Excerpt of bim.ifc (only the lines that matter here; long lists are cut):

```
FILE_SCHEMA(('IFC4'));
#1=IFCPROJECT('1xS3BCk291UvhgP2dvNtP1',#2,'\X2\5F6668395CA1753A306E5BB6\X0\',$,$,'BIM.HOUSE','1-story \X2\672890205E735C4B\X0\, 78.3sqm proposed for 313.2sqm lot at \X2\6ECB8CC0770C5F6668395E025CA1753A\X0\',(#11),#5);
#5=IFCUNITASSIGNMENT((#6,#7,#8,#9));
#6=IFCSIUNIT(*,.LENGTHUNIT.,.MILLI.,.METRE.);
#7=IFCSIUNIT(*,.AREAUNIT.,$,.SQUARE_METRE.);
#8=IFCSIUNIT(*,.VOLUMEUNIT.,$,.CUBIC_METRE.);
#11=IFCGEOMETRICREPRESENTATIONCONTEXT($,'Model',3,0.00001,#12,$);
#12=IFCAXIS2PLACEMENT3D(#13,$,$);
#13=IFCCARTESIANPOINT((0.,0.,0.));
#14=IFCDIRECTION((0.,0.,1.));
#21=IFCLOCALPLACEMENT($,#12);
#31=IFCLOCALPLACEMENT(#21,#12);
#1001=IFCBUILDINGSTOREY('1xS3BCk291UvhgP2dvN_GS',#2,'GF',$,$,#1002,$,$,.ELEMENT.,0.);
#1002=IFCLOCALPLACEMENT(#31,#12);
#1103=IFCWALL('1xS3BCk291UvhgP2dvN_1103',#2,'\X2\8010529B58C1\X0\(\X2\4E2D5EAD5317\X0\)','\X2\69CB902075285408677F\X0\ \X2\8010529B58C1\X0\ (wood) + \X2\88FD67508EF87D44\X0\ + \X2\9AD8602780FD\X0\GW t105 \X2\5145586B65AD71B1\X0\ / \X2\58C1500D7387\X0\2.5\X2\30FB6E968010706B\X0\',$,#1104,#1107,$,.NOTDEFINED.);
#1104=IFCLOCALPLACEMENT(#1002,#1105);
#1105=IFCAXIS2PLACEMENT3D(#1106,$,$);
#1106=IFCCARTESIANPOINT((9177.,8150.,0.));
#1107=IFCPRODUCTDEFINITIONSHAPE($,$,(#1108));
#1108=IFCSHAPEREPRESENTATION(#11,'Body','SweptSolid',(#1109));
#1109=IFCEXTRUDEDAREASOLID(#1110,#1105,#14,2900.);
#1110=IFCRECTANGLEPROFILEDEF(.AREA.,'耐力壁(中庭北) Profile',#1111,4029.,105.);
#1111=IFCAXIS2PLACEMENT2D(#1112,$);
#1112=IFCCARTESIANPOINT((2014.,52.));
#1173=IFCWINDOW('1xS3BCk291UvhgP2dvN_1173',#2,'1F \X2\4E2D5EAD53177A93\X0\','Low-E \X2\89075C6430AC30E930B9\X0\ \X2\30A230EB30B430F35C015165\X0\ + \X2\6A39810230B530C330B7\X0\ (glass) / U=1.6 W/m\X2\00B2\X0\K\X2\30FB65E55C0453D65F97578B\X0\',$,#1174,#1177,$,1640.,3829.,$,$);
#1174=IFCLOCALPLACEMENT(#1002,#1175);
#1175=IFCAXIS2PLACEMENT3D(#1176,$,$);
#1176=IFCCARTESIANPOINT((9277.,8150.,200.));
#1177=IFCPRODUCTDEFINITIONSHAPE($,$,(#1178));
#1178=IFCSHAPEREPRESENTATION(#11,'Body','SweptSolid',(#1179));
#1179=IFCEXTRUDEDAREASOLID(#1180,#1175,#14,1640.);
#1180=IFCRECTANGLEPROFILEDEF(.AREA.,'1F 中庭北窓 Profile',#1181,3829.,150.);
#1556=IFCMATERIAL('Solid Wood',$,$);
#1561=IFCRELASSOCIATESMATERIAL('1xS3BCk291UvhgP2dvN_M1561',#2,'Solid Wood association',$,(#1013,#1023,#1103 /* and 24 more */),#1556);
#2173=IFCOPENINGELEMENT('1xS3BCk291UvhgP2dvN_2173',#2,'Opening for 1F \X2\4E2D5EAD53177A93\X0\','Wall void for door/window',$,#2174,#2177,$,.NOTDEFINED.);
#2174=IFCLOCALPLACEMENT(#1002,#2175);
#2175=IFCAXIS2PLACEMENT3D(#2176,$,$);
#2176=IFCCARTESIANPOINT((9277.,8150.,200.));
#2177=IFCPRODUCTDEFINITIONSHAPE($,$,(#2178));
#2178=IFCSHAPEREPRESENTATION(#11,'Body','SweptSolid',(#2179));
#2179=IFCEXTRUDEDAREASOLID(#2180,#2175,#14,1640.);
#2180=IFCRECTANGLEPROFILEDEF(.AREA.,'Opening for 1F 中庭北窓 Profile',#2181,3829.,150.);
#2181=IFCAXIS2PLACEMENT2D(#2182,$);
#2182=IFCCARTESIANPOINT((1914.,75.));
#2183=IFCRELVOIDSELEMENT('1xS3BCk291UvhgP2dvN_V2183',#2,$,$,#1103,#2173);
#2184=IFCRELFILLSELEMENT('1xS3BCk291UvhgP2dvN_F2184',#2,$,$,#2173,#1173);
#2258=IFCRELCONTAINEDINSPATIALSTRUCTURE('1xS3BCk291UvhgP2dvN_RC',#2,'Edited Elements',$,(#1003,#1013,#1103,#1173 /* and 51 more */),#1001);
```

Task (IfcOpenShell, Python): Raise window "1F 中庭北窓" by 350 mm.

```python
import numpy as np
import ifcopenshell
import ifcopenshell.api.geometry
import ifcopenshell.util.placement
import ifcopenshell.util.unit

model = ifcopenshell.open("bim.ifc")
unit_scale = ifcopenshell.util.unit.calculate_unit_scale(model)

window = model.by_guid("1xS3BCk291UvhgP2dvN_1173")
opening = window.FillsVoids[0].RelatingOpeningElement
dz = 0.35 / unit_scale

shift = np.array([0.0, 0.0, dz])
# The window is not placed relative to its opening, so move both.
for product in (opening, window):
    matrix = ifcopenshell.util.placement.get_local_placement(product.ObjectPlacement)
    matrix[:3, 3] += shift
    ifcopenshell.api.geometry.edit_object_placement(model, product=product, matrix=matrix, is_si=False)

print(f"moved by {dz * unit_scale:+.3f} m")

model.write("bim_edited.ifc")
```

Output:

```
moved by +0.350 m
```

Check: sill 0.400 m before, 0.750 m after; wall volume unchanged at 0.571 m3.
